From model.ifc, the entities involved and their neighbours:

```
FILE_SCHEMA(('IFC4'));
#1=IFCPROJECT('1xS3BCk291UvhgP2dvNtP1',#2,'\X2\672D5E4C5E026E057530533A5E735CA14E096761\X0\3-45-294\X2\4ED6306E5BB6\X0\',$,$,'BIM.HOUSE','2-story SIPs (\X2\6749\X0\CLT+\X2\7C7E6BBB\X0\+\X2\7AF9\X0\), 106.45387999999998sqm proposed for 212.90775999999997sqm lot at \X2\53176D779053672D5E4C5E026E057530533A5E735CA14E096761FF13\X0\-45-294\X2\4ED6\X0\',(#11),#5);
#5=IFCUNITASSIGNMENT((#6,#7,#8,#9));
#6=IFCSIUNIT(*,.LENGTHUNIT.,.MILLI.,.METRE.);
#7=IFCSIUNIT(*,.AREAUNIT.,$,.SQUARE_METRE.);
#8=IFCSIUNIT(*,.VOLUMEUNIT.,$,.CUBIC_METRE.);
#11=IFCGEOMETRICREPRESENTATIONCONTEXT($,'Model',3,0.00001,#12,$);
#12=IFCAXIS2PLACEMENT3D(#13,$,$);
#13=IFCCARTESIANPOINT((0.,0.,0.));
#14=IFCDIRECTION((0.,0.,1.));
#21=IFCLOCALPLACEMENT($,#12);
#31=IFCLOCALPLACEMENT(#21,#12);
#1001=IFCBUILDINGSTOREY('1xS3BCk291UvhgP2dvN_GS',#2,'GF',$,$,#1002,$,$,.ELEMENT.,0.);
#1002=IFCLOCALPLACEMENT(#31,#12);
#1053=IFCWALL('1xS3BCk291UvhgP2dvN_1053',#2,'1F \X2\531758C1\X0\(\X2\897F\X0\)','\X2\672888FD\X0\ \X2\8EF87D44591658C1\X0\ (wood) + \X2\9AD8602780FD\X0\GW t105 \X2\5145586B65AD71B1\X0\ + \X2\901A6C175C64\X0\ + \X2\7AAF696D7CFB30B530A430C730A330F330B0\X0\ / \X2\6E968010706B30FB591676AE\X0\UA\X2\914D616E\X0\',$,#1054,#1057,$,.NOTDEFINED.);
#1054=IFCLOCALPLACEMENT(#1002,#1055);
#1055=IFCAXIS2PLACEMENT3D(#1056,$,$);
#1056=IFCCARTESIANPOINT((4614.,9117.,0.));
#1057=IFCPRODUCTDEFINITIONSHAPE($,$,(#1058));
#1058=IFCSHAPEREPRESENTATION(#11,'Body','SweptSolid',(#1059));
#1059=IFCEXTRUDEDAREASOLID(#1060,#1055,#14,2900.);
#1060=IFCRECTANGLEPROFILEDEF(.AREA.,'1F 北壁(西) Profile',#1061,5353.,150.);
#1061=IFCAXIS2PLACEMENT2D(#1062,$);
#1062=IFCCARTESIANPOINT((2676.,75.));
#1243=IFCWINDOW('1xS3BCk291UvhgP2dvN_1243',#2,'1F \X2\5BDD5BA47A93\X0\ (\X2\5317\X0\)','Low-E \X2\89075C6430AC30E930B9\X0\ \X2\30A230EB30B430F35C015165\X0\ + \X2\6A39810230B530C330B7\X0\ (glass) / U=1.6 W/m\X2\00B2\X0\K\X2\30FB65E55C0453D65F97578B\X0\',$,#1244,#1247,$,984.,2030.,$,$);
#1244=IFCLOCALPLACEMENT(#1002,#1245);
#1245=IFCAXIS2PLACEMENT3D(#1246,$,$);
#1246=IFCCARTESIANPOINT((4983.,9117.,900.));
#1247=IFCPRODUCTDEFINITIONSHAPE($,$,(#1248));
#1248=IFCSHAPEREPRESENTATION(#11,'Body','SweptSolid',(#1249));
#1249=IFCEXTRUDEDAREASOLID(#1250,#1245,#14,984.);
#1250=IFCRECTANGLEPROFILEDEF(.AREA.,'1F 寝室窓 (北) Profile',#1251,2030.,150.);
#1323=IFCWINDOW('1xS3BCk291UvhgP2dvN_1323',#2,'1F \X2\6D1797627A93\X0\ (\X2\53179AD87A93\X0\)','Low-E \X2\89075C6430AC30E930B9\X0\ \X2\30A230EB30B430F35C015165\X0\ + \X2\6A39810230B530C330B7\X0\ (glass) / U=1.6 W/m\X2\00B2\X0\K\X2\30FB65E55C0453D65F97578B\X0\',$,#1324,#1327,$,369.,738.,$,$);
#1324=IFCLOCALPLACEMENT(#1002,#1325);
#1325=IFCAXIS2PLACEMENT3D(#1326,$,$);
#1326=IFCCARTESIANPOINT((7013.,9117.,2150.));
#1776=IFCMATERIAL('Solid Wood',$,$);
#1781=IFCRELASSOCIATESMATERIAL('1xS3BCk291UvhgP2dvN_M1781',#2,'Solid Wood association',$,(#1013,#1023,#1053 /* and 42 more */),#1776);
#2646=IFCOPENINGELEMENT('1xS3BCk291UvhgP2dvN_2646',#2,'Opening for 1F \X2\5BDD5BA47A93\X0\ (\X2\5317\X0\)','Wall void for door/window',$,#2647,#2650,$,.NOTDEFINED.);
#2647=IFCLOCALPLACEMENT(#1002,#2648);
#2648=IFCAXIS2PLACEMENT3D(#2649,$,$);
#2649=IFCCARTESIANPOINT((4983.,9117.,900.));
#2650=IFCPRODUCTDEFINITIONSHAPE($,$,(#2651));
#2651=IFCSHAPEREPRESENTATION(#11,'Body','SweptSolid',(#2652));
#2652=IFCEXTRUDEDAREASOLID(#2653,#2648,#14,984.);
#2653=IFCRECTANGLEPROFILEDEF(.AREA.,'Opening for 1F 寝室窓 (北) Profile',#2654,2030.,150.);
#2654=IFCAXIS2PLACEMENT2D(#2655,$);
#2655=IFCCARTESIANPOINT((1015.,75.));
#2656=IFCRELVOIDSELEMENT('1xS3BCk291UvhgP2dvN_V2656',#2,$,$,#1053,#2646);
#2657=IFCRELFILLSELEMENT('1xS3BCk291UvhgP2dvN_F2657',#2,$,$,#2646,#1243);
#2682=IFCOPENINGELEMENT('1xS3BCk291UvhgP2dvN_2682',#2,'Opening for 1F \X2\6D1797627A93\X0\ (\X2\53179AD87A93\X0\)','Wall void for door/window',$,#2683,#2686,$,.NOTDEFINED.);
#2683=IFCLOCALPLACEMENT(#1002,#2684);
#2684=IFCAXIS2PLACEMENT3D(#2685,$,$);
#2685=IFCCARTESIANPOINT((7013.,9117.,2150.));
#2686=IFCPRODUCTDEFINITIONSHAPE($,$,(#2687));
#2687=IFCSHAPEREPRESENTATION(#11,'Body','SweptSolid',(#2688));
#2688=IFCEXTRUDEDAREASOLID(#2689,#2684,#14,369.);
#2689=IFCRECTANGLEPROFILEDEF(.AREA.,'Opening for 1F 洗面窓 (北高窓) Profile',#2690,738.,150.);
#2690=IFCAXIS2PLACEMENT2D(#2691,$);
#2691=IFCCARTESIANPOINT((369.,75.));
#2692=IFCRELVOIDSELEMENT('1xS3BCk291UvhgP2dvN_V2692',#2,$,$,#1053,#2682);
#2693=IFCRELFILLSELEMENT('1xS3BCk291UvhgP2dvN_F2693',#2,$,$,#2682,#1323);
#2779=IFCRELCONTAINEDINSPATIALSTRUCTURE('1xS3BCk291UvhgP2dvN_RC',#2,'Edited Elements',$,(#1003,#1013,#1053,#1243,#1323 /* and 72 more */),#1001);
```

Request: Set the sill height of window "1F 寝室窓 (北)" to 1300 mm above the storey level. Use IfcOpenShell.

```python
import numpy as np
import ifcopenshell
import ifcopenshell.api.geometry
import ifcopenshell.geom
import ifcopenshell.util.element
import ifcopenshell.util.placement
import ifcopenshell.util.shape
import ifcopenshell.util.unit

model = ifcopenshell.open("model.ifc")
unit_scale = ifcopenshell.util.unit.calculate_unit_scale(model)

window = model.by_id(1243)
opening = window.FillsVoids[0].RelatingOpeningElement
storey = ifcopenshell.util.element.get_container(window, ifc_class="IfcBuildingStorey")
level = ifcopenshell.util.placement.get_local_placement(storey.ObjectPlacement)[2, 3]

# The opening's origin need not be at the sill, so measure its lowest point.
shape = ifcopenshell.geom.create_shape(ifcopenshell.geom.settings(), opening)
bottom = ifcopenshell.util.shape.get_shape_bottom_elevation(shape, shape.geometry) / unit_scale
dz = level + 1300.0 - bottom

shift = np.array([0.0, 0.0, dz])
# The window is not placed relative to its opening, so move both.
for product in (opening, window):
    matrix = ifcopenshell.util.placement.get_local_placement(product.ObjectPlacement)
    matrix[:3, 3] += shift
    ifcopenshell.api.geometry.edit_object_placement(model, product=product, matrix=matrix, is_si=False)

print(f"moved by {dz * unit_scale:+.3f} m")

model.write("model_updated.ifc")
```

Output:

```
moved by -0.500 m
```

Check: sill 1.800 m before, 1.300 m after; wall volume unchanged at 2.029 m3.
